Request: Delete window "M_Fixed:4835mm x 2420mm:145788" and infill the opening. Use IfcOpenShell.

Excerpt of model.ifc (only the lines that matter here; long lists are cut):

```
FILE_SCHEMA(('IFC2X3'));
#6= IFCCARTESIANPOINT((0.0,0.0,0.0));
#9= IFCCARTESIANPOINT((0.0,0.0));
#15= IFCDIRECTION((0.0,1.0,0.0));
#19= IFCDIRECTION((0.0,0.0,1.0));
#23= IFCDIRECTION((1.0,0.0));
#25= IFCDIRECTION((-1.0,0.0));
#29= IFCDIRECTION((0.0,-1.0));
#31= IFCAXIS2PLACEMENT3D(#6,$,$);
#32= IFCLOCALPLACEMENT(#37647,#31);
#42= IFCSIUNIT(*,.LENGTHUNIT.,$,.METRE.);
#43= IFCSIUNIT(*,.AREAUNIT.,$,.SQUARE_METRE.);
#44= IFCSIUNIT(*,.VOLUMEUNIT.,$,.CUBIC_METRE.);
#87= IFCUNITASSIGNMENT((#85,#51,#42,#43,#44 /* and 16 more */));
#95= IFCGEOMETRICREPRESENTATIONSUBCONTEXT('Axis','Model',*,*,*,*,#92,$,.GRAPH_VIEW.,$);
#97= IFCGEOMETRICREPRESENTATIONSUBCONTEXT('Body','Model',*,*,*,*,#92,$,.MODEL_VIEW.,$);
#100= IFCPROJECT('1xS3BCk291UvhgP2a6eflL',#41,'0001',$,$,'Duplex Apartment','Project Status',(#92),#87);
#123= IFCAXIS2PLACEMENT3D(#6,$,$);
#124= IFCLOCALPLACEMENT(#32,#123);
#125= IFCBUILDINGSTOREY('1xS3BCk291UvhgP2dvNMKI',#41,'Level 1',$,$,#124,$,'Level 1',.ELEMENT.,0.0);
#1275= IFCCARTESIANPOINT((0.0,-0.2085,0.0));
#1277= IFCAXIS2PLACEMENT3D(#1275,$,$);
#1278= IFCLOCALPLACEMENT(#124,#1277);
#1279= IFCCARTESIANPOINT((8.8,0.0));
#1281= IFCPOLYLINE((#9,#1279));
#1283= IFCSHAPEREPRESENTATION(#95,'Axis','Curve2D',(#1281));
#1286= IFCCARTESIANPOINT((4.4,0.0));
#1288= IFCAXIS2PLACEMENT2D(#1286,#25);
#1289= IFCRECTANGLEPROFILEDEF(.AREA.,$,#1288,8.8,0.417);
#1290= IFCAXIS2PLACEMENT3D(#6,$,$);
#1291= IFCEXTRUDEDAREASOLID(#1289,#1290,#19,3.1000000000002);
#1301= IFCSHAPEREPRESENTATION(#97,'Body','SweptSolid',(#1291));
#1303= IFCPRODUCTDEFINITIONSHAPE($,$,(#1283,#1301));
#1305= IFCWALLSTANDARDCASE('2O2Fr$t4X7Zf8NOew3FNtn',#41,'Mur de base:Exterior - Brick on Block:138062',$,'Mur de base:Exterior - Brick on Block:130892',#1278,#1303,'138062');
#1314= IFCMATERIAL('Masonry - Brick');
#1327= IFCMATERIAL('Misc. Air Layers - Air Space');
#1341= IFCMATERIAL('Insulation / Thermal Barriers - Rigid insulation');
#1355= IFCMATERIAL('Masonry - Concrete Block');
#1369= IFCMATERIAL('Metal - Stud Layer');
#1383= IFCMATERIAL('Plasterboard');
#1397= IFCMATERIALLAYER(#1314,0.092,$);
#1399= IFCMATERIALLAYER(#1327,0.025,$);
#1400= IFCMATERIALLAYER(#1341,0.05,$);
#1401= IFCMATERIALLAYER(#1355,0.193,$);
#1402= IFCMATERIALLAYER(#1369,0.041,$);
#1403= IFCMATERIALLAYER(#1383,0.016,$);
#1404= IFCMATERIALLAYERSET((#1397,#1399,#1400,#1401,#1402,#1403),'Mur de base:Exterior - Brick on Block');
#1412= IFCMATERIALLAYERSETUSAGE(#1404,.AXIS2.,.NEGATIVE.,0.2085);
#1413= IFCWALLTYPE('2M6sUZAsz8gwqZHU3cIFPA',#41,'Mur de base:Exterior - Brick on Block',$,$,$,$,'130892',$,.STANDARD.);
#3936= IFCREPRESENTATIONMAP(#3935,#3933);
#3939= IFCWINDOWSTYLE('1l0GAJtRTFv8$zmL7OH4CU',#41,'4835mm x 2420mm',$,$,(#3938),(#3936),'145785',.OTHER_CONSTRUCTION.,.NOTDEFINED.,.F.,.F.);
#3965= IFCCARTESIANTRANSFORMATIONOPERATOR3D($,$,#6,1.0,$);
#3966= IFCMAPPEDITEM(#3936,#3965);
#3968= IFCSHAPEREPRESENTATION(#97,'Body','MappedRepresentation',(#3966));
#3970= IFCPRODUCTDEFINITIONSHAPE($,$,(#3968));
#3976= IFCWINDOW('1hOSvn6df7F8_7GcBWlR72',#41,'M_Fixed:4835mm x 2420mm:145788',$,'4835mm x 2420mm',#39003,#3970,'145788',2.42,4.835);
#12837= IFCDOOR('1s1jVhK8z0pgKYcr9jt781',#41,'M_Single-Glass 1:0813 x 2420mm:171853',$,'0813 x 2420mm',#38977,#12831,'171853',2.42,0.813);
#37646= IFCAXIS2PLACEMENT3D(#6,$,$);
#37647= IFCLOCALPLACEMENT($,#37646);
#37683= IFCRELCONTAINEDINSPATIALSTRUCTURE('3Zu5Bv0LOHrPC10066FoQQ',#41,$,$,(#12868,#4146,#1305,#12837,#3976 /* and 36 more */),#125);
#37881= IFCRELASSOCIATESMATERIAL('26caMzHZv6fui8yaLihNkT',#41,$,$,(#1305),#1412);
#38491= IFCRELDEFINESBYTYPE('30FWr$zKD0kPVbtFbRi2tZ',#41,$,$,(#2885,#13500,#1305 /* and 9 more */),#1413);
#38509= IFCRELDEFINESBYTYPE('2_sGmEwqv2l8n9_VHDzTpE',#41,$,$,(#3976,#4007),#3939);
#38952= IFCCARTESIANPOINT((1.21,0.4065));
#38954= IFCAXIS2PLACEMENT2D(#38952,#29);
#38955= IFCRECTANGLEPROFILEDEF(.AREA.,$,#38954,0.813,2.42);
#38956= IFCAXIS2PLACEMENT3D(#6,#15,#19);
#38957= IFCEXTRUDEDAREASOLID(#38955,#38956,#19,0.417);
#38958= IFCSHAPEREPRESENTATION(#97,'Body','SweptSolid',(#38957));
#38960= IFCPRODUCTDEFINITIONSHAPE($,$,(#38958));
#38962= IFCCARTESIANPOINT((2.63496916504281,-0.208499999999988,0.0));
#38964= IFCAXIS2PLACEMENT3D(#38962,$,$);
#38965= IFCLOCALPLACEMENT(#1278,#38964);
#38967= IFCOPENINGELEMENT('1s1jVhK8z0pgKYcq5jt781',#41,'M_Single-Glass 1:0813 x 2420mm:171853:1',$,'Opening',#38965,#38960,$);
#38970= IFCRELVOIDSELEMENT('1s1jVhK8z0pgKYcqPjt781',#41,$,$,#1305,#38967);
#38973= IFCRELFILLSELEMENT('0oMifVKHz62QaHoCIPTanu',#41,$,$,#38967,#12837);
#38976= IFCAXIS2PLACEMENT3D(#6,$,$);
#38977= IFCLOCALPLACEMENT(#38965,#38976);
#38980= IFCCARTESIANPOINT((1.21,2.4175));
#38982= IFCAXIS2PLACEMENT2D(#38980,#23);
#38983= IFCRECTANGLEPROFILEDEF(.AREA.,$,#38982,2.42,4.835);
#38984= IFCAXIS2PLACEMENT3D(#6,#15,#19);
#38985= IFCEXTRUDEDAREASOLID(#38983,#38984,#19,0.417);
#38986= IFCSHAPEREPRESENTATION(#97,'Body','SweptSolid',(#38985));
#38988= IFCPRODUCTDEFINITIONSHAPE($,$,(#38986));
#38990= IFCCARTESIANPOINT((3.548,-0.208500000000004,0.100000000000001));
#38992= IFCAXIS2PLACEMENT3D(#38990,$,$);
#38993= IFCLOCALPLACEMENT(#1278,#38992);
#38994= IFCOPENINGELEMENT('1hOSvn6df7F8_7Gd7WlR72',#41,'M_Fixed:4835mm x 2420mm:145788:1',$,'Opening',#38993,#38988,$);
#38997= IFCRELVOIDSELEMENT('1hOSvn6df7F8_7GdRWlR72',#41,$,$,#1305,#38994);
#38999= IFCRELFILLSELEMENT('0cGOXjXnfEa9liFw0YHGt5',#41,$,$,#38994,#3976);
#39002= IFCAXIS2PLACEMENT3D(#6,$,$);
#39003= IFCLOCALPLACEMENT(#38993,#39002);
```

```python
import ifcopenshell
import ifcopenshell.api.feature
import ifcopenshell.api.root
import ifcopenshell.geom
import ifcopenshell.util.shape

model = ifcopenshell.open("model.ifc")
settings = ifcopenshell.geom.settings()


def volume(element):
    """Net volume in cubic metres, openings subtracted."""
    shape = ifcopenshell.geom.create_shape(settings, element)
    return ifcopenshell.util.shape.get_volume(shape.geometry)


window = model.by_id(3976)
opening = window.FillsVoids[0].RelatingOpeningElement
wall = opening.VoidsElements[0].RelatingBuildingElement
before = volume(wall)

ifcopenshell.api.root.remove_product(model, product=window)
ifcopenshell.api.feature.remove_feature(model, feature=opening)

after = volume(wall)

print(f"wall volume {before:.3f} -> {after:.3f} m3")

model.write("model_rev.ifc")
```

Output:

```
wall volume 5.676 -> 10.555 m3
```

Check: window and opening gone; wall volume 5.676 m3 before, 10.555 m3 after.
